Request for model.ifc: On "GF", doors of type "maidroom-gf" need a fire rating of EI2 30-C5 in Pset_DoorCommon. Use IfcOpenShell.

First a look at what the model holds.

```python
import ifcopenshell
import ifcopenshell.util.element

model = ifcopenshell.open("model.ifc")
print(model.schema)
storey = next(s for s in model.by_type("IfcBuildingStorey") if s.Name == "GF")
doors = [e for e in ifcopenshell.util.element.get_decomposition(storey) if e.is_a("IfcDoor")]
seen = {}
for e in doors:
    element_type = ifcopenshell.util.element.get_type(e)
    key = (element_type.Name if element_type != e and element_type else None, ifcopenshell.util.element.get_pset(e, "Pset_DoorCommon", "FireRating"))
    seen[key] = seen.get(key, 0) + 1
for (name, value), count in sorted(seen.items(), key=str):
    print(count, "x", name, "|", value)
```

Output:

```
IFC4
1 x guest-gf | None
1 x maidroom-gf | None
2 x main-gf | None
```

```python
import ifcopenshell
import ifcopenshell.api.pset
import ifcopenshell.util.element

model = ifcopenshell.open("model.ifc")

storey = next(s for s in model.by_type("IfcBuildingStorey") if s.Name == "GF")
doors = [e for e in ifcopenshell.util.element.get_decomposition(storey) if e.is_a("IfcDoor")]

count = 0
for e in doors:
    element_type = ifcopenshell.util.element.get_type(e)
    if element_type in (None, e) or element_type.Name != "maidroom-gf":
        continue
    # add_pset returns the element's existing set when there is one.
    pset = ifcopenshell.api.pset.add_pset(model, product=e, name="Pset_DoorCommon")
    ifcopenshell.api.pset.edit_pset(model, pset=pset, properties={"FireRating": "EI2 30-C5"})
    count += 1

print(count, "doors updated")

model.write("model_updated.ifc")
```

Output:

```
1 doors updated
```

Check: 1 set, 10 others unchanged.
